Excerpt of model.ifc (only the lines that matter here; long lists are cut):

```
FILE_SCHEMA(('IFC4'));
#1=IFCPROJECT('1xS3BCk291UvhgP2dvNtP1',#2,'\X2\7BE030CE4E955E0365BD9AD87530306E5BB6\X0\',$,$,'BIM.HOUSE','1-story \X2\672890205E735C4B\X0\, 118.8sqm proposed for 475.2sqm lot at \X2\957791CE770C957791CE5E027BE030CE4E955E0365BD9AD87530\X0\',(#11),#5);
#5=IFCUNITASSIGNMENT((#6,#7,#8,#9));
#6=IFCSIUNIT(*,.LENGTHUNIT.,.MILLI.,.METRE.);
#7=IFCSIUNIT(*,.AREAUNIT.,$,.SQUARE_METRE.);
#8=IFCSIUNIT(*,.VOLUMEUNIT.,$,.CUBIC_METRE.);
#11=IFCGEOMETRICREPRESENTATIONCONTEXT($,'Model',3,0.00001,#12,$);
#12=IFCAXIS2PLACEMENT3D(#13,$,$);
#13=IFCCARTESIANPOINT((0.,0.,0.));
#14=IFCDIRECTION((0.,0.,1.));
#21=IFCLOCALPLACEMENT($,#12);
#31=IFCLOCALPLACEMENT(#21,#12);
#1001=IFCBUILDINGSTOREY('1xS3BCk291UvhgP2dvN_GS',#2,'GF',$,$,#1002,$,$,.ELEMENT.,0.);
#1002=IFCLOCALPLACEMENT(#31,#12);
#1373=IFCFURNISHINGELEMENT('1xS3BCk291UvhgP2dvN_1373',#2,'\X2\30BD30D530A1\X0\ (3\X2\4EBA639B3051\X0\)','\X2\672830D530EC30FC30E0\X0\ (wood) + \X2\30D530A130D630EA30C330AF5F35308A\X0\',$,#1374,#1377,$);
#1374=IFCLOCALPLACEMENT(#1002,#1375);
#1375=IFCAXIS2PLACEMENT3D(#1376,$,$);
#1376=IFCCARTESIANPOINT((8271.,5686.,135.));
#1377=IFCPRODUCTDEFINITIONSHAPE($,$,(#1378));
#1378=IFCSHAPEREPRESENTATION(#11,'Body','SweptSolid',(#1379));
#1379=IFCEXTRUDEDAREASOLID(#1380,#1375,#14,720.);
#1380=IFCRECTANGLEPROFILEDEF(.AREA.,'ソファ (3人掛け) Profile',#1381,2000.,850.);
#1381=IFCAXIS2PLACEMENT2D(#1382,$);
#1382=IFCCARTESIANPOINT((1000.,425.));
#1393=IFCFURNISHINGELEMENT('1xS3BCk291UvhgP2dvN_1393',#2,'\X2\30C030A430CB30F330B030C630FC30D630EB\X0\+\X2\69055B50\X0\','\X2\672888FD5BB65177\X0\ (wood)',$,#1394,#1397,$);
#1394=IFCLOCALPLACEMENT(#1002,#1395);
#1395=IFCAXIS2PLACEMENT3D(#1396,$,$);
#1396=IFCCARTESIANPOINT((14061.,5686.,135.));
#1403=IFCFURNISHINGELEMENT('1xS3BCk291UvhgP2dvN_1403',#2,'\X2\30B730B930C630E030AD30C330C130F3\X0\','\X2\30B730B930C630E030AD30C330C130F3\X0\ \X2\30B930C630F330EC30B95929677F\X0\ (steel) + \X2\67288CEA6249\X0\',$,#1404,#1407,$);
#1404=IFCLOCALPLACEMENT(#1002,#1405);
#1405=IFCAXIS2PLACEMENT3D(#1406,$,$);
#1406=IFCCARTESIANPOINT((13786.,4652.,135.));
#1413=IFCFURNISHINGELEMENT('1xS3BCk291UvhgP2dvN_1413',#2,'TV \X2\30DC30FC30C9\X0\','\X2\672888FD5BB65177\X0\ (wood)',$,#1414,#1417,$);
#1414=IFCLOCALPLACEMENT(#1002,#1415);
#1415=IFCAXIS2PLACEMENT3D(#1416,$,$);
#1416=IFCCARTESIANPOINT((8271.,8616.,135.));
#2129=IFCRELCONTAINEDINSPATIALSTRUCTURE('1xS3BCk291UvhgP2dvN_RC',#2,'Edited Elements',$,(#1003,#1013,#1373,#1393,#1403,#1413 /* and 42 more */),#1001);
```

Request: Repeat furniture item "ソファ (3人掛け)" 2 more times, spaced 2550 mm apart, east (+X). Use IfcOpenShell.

```python
import numpy as np
import ifcopenshell
import ifcopenshell.api.geometry
import ifcopenshell.api.root
import ifcopenshell.util.element
import ifcopenshell.util.placement
import ifcopenshell.util.unit

model = ifcopenshell.open("model.ifc")
unit_scale = ifcopenshell.util.unit.calculate_unit_scale(model)


def reuse_history(source, copy):
    """copy_class also copies each property set's owner history, people and application; keep the originals."""
    for rel in copy.IsDefinedBy:
        if rel.is_a("IfcRelDefinesByProperties") and (history := rel.RelatingPropertyDefinition.OwnerHistory):
            rel.RelatingPropertyDefinition.OwnerHistory = source.OwnerHistory
            ifcopenshell.util.element.remove_deep2(model, history)


source = model.by_guid("1xS3BCk291UvhgP2dvN_1373")
base = ifcopenshell.util.placement.get_local_placement(source.ObjectPlacement)
step = np.array([1.0, 0.0, 0.0]) * 2.55 / unit_scale

for i in range(1, 3):
    copy = ifcopenshell.api.root.copy_class(model, product=source)
    copy.Representation = ifcopenshell.util.element.copy_deep(
        model, source.Representation, exclude=["IfcGeometricRepresentationContext", "IfcRepresentationMap"]
    )
    reuse_history(source, copy)
    matrix = base.copy()
    matrix[:3, 3] += i * step
    print("added at", matrix[:3, 3].round(3) + 0.0)
    ifcopenshell.api.geometry.edit_object_placement(model, product=copy, matrix=matrix, is_si=False)

model.write("model_updated.ifc")
```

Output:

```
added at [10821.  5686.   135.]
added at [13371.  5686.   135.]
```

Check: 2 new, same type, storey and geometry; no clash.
